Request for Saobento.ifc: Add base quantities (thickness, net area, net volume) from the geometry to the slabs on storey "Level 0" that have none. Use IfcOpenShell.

First a look at what the model holds.

```python
import ifcopenshell
import ifcopenshell.util.element
import ifcopenshell.util.unit

model = ifcopenshell.open("Saobento.ifc")
print(model.schema)
for unit_type in ("LENGTHUNIT", "AREAUNIT", "VOLUMEUNIT"):
    print(unit_type, ifcopenshell.util.unit.calculate_unit_scale(model, unit_type))
storey = next(s for s in model.by_type("IfcBuildingStorey") if s.Name == "Level 0")
slabs = [e for e in ifcopenshell.util.element.get_decomposition(storey) if e.is_a("IfcSlab")]
for e in sorted(slabs, key=lambda e: e.id()):
    print(e.id(), e.is_a(), e.Name, list(ifcopenshell.util.element.get_psets(e, qtos_only=True)), sep=" | ")
```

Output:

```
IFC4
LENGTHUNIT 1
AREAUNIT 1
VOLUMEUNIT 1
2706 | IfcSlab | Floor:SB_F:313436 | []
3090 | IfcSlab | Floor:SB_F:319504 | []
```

```python
import ifcopenshell
import ifcopenshell.api.pset
import ifcopenshell.geom
import ifcopenshell.util.element
import ifcopenshell.util.shape
import ifcopenshell.util.unit

model = ifcopenshell.open("Saobento.ifc")
unit_scale = ifcopenshell.util.unit.calculate_unit_scale(model)
area_scale = ifcopenshell.util.unit.calculate_unit_scale(model, "AREAUNIT")
volume_scale = ifcopenshell.util.unit.calculate_unit_scale(model, "VOLUMEUNIT")
settings = ifcopenshell.geom.settings()

storey = next(s for s in model.by_type("IfcBuildingStorey") if s.Name == "Level 0")
slabs = [e for e in ifcopenshell.util.element.get_decomposition(storey) if e.is_a("IfcSlab")]

for e in sorted(slabs, key=lambda e: e.id()):
    if ifcopenshell.util.element.get_psets(e, qtos_only=True, should_inherit=False):
        continue
    # Geometry comes back in metres, in the element's own axes.
    shape = ifcopenshell.geom.create_shape(settings, e)
    values = {
        "Width": ifcopenshell.util.shape.get_z(shape.geometry) / unit_scale,
        "NetArea": ifcopenshell.util.shape.get_footprint_area(shape.geometry) / area_scale,
        "NetVolume": ifcopenshell.util.shape.get_volume(shape.geometry) / volume_scale,
    }
    qto = ifcopenshell.api.pset.add_qto(model, product=e, name="Qto_SlabBaseQuantities")
    ifcopenshell.api.pset.edit_qto(model, qto=qto, properties=values)
    print(e.id(), {k: round(v, 3) for k, v in values.items()})

model.write("Saobento_edited.ifc")
```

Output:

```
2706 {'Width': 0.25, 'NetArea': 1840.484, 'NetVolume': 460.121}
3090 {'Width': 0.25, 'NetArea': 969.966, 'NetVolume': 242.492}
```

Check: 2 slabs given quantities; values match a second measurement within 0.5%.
